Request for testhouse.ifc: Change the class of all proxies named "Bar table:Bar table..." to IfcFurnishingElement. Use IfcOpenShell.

First a look at what the model holds.

```python
import re

import ifcopenshell

model = ifcopenshell.open("testhouse.ifc")
print(model.schema)
seen = {}
for e in model.by_type("IfcBuildingElementProxy"):
    name = re.sub(r":\d+(:\d+)?$", "", e.Name or "")  # drop the element id that some exporters append
    seen[name] = seen.get(name, 0) + 1
for name, count in sorted(seen.items()):
    print(count, "x", name)
```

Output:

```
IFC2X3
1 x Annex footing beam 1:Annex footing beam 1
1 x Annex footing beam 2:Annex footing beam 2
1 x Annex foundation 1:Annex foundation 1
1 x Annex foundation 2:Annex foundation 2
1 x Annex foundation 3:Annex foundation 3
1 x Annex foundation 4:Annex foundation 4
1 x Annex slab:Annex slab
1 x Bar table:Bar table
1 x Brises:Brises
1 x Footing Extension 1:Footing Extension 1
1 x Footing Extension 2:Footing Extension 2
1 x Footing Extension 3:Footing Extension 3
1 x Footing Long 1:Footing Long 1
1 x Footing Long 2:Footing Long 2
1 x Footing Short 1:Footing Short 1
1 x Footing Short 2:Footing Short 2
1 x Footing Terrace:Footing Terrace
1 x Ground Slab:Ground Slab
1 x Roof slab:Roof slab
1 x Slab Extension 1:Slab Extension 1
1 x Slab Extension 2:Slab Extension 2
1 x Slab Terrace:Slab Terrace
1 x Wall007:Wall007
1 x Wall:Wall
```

```python
import ifcopenshell
import ifcopenshell.api.root

model = ifcopenshell.open("testhouse.ifc")

proxies = [e.id() for e in model.by_type("IfcBuildingElementProxy") if (e.Name or "").startswith("Bar table:Bar table")]
for step_id in proxies:
    proxy = model.by_id(step_id)
    ifcopenshell.api.root.reassign_class(model, product=proxy, ifc_class="IfcFurnishingElement")

print(sum(model.by_id(i).is_a("IfcFurnishingElement") for i in proxies), "reclassified")

model.write("testhouse_updated.ifc")
```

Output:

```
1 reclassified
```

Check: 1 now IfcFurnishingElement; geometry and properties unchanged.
